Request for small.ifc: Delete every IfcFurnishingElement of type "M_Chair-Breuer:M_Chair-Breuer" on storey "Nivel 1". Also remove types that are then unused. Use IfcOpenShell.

First a look at what the model holds.

```python
import ifcopenshell
import ifcopenshell.util.element

model = ifcopenshell.open("small.ifc")
print(model.schema)
storey = next(s for s in model.by_type("IfcBuildingStorey") if s.Name == "Nivel 1")
furniture = [e for e in ifcopenshell.util.element.get_decomposition(storey) if e.is_a("IfcFurnishingElement")]
seen = {}
for e in furniture:
    element_type = ifcopenshell.util.element.get_type(e)
    name = element_type.Name if element_type not in (None, e) else None
    seen[name] = seen.get(name, 0) + 1
for name, count in sorted(seen.items(), key=str):
    print(count, "x", name)
```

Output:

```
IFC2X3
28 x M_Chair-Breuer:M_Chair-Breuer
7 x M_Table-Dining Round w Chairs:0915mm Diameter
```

```python
import ifcopenshell
import ifcopenshell.api.root
import ifcopenshell.util.element

model = ifcopenshell.open("small.ifc")

storey = next(s for s in model.by_type("IfcBuildingStorey") if s.Name == "Nivel 1")
furniture = [e for e in ifcopenshell.util.element.get_decomposition(storey) if e.is_a("IfcFurnishingElement")]
targets = [e for e in furniture if (t := ifcopenshell.util.element.get_type(e)) not in (None, e) and t.Name == "M_Chair-Breuer:M_Chair-Breuer"]
types = {ifcopenshell.util.element.get_type(e) for e in targets} - {None, *targets}

for e in targets:
    ifcopenshell.api.root.remove_product(model, product=e)
print(len(targets), "removed")

unused = [t for t in types if not ifcopenshell.util.element.get_types(t)]
for t in unused:
    ifcopenshell.api.root.remove_product(model, product=t)
print(len(unused), "unused types removed")

model.write("small_edited.ifc")
```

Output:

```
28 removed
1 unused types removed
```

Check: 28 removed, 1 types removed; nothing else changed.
